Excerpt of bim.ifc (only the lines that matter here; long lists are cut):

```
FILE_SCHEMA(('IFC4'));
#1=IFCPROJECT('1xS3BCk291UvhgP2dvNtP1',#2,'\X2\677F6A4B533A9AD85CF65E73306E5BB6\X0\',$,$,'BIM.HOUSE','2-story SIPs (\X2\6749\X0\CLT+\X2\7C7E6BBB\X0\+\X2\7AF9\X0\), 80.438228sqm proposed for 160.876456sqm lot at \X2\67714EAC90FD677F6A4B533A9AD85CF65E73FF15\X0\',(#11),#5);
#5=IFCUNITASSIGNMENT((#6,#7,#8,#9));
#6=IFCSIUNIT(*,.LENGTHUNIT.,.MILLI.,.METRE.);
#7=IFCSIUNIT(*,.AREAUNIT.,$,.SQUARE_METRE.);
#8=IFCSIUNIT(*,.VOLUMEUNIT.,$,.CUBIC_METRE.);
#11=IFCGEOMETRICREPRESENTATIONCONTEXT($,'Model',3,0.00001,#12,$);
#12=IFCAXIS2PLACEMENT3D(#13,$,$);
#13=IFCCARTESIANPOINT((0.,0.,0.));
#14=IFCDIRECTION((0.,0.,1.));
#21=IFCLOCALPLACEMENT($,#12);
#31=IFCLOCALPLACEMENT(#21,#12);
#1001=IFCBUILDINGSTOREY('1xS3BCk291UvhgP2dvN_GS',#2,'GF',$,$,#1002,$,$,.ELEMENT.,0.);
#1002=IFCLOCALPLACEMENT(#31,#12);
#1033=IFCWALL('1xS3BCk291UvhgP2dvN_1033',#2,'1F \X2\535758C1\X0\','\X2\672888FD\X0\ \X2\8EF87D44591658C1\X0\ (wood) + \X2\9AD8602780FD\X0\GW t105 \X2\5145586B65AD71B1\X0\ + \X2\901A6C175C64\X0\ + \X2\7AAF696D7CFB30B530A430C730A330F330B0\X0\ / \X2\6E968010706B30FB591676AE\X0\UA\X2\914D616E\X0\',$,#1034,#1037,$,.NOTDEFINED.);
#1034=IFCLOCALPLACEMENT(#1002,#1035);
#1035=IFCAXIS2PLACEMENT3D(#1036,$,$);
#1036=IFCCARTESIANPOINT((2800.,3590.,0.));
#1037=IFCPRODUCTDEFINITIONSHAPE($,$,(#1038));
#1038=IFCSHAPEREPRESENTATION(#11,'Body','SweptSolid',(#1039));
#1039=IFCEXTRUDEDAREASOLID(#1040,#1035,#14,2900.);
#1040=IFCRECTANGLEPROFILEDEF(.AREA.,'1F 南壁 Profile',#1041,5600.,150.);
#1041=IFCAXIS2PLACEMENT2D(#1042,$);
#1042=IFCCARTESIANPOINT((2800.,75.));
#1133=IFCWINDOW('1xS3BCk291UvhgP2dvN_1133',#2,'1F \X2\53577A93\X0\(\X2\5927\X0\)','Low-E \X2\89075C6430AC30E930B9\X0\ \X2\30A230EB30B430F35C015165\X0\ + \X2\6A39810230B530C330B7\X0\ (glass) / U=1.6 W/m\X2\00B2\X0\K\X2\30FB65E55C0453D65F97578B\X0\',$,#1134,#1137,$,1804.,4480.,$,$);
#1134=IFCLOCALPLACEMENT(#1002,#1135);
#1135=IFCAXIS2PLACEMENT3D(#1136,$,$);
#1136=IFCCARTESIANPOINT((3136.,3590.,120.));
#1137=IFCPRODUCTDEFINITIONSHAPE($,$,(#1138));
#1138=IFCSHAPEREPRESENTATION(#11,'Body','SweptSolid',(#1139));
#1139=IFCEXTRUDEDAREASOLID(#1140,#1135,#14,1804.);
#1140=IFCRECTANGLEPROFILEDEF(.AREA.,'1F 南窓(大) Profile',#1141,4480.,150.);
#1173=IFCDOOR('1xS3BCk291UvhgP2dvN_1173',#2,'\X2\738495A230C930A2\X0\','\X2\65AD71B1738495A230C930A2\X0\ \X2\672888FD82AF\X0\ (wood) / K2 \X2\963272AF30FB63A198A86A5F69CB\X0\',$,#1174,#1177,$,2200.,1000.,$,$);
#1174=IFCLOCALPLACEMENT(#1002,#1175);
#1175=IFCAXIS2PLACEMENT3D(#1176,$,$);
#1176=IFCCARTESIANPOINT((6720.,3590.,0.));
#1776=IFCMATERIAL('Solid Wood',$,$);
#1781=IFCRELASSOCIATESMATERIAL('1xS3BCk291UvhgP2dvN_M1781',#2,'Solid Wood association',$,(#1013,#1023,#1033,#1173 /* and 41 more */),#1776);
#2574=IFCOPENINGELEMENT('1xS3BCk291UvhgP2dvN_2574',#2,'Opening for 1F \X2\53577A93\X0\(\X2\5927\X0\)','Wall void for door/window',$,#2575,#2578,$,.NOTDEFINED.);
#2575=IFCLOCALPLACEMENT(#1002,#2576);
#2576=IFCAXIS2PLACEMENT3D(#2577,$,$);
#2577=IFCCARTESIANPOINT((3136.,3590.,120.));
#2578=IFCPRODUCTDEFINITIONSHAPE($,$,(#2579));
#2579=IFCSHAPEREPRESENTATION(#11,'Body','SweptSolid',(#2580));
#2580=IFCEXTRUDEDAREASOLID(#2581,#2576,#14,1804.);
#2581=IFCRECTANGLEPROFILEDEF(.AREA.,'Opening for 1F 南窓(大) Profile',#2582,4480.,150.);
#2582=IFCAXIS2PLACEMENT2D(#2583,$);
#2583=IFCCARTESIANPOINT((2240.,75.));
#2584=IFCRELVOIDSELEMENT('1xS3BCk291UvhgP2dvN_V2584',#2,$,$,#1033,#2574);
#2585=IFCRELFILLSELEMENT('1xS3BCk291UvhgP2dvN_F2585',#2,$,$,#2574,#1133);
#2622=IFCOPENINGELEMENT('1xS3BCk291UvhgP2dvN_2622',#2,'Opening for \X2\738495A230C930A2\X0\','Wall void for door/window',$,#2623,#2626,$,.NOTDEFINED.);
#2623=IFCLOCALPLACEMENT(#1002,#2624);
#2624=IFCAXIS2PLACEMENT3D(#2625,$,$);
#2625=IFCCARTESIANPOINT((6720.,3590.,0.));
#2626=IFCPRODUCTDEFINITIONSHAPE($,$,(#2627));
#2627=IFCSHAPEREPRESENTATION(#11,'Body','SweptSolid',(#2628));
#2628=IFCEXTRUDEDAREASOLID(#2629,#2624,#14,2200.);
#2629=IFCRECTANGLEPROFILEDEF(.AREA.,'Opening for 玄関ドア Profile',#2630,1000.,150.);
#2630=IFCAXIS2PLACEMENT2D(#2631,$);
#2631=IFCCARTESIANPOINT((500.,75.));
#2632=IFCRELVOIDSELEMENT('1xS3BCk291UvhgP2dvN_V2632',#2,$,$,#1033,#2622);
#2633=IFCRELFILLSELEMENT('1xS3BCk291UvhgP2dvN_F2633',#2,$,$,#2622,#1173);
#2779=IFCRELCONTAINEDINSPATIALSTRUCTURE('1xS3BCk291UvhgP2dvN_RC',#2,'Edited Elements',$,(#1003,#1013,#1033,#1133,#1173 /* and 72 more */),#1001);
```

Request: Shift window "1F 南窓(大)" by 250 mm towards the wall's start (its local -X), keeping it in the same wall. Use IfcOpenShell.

```python
import ifcopenshell
import ifcopenshell.api.geometry
import ifcopenshell.util.placement

model = ifcopenshell.open("bim.ifc")

window = model.by_guid("1xS3BCk291UvhgP2dvN_1133")
opening = window.FillsVoids[0].RelatingOpeningElement
wall = opening.VoidsElements[0].RelatingBuildingElement

wall_matrix = ifcopenshell.util.placement.get_local_placement(wall.ObjectPlacement)
shift = wall_matrix[:3, 0] * -250.0
before = ifcopenshell.util.placement.get_local_placement(window.ObjectPlacement)[:3, 3].copy()

# The window is not placed relative to its opening, so move both.
for product in (opening, window):
    matrix = ifcopenshell.util.placement.get_local_placement(product.ObjectPlacement)
    matrix[:3, 3] += shift
    ifcopenshell.api.geometry.edit_object_placement(model, product=product, matrix=matrix, is_si=False)

after = ifcopenshell.util.placement.get_local_placement(window.ObjectPlacement)[:3, 3]
print("window moved by", (after - before).round(3) + 0.0)

model.write("bim_updated.ifc")
```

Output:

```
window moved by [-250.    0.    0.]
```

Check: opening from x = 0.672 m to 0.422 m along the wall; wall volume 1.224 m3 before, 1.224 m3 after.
